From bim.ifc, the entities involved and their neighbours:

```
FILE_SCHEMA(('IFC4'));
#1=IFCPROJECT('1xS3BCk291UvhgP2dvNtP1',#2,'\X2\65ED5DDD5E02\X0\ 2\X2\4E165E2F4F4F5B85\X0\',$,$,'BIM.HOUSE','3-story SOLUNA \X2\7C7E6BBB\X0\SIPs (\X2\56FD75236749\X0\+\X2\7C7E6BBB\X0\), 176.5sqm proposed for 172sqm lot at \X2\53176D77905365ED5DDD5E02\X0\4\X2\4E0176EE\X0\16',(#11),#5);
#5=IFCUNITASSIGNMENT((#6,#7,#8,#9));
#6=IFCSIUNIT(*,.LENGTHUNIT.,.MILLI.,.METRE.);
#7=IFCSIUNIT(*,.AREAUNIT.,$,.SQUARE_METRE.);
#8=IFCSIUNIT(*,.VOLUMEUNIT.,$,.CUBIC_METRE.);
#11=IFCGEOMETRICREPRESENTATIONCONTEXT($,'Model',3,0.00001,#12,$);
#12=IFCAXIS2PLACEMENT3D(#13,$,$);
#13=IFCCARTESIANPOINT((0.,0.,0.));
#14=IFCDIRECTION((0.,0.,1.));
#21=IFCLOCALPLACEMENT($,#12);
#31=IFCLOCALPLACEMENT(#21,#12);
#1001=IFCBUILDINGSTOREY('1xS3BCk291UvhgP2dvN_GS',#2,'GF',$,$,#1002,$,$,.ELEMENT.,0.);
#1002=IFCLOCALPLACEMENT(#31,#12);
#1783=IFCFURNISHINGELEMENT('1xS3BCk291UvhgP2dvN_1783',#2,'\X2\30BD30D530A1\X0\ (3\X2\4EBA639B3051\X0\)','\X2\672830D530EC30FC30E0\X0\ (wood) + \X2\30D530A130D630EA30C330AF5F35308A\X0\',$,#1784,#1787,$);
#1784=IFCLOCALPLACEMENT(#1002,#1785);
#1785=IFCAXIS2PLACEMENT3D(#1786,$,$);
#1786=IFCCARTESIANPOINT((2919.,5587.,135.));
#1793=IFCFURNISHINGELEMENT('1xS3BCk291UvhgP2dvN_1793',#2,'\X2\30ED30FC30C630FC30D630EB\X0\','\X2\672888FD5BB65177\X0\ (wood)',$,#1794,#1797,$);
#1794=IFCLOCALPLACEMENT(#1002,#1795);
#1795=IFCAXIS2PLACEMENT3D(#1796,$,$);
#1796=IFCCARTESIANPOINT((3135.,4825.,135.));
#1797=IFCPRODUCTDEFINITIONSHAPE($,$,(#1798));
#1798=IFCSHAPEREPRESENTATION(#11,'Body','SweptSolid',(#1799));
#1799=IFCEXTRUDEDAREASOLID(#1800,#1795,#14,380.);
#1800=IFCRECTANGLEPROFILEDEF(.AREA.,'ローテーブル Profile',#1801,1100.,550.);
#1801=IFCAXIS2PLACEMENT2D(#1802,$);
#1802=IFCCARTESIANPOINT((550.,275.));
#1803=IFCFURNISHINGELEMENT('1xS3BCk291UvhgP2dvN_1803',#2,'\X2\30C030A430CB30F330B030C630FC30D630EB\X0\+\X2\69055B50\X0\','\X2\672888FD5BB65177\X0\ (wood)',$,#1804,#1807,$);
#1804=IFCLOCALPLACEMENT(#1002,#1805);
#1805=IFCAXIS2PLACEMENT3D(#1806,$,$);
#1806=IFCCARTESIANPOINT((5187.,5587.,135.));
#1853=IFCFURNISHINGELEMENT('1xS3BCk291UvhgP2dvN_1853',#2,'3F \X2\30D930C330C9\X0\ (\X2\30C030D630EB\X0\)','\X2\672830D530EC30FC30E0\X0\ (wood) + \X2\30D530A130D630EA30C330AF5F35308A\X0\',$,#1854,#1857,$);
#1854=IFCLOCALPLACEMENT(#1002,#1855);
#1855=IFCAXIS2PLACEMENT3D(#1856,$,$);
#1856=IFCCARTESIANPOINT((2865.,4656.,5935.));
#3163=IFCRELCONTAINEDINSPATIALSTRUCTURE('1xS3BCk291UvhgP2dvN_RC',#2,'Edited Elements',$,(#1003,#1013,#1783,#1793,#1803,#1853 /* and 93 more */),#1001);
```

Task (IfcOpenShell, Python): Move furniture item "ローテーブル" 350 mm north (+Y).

```python
import ifcopenshell
import ifcopenshell.api.geometry
import ifcopenshell.util.placement
import ifcopenshell.util.unit

model = ifcopenshell.open("bim.ifc")
unit_scale = ifcopenshell.util.unit.calculate_unit_scale(model)

item = model.by_guid("1xS3BCk291UvhgP2dvN_1793")
matrix = ifcopenshell.util.placement.get_local_placement(item.ObjectPlacement)
matrix[1, 3] += 0.35 / unit_scale
ifcopenshell.api.geometry.edit_object_placement(model, product=item, matrix=matrix, is_si=False)

print(ifcopenshell.util.placement.get_local_placement(item.ObjectPlacement).round(3) + 0.0)

model.write("bim_edited.ifc")
```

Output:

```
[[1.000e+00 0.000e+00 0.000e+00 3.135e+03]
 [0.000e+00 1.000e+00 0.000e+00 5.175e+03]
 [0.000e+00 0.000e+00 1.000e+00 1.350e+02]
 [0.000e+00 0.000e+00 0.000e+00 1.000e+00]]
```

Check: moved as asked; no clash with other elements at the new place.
